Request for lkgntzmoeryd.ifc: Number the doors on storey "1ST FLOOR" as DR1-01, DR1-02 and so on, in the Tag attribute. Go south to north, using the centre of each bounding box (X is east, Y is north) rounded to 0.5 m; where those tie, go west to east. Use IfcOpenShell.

First a look at what the model holds.

```python
import ifcopenshell
import ifcopenshell.util.element
import ifcopenshell.util.placement

model = ifcopenshell.open("lkgntzmoeryd.ifc")
print(model.schema)
storey = next(s for s in model.by_type("IfcBuildingStorey") if s.Name == "1ST FLOOR")
doors = [e for e in ifcopenshell.util.element.get_decomposition(storey) if e.is_a("IfcDoor")]
for e in sorted(doors, key=lambda e: e.id()):
    origin = ifcopenshell.util.placement.get_local_placement(e.ObjectPlacement)[:3, 3]
    print(e.id(), e.Tag, e.Name, origin.round(2) + 0.0, sep=" | ")
```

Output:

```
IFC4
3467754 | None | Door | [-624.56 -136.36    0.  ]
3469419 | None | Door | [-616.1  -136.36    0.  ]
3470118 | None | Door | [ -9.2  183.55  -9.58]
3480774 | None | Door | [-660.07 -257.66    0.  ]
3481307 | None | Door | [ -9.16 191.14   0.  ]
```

```python
import ifcopenshell
import ifcopenshell.geom
import ifcopenshell.util.element
import ifcopenshell.util.shape

model = ifcopenshell.open("lkgntzmoeryd.ifc")
settings = ifcopenshell.geom.settings()
settings.set("use-world-coords", True)


def centre(element):
    shape = ifcopenshell.geom.create_shape(settings, element)
    return ifcopenshell.util.shape.get_bbox_centroid(shape.geometry)


storey = next(s for s in model.by_type("IfcBuildingStorey") if s.Name == "1ST FLOOR")
doors = [e for e in ifcopenshell.util.element.get_decomposition(storey) if e.is_a("IfcDoor")]

# Insertion points can sit at a corner or the storey origin, so sort by the geometry (in metres).
centres = {e: centre(e) for e in doors}
doors.sort(key=lambda e: (round(centres[e][1] / 0.5), centres[e][0]))

for i, e in enumerate(doors, start=1):
    number = f"DR1-{i:02d}"
    e.Tag = number
    print(e.id(), number)

model.write("lkgntzmoeryd_v2.ifc")
```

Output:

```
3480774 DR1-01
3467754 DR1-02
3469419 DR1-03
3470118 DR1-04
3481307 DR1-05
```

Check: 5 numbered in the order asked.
